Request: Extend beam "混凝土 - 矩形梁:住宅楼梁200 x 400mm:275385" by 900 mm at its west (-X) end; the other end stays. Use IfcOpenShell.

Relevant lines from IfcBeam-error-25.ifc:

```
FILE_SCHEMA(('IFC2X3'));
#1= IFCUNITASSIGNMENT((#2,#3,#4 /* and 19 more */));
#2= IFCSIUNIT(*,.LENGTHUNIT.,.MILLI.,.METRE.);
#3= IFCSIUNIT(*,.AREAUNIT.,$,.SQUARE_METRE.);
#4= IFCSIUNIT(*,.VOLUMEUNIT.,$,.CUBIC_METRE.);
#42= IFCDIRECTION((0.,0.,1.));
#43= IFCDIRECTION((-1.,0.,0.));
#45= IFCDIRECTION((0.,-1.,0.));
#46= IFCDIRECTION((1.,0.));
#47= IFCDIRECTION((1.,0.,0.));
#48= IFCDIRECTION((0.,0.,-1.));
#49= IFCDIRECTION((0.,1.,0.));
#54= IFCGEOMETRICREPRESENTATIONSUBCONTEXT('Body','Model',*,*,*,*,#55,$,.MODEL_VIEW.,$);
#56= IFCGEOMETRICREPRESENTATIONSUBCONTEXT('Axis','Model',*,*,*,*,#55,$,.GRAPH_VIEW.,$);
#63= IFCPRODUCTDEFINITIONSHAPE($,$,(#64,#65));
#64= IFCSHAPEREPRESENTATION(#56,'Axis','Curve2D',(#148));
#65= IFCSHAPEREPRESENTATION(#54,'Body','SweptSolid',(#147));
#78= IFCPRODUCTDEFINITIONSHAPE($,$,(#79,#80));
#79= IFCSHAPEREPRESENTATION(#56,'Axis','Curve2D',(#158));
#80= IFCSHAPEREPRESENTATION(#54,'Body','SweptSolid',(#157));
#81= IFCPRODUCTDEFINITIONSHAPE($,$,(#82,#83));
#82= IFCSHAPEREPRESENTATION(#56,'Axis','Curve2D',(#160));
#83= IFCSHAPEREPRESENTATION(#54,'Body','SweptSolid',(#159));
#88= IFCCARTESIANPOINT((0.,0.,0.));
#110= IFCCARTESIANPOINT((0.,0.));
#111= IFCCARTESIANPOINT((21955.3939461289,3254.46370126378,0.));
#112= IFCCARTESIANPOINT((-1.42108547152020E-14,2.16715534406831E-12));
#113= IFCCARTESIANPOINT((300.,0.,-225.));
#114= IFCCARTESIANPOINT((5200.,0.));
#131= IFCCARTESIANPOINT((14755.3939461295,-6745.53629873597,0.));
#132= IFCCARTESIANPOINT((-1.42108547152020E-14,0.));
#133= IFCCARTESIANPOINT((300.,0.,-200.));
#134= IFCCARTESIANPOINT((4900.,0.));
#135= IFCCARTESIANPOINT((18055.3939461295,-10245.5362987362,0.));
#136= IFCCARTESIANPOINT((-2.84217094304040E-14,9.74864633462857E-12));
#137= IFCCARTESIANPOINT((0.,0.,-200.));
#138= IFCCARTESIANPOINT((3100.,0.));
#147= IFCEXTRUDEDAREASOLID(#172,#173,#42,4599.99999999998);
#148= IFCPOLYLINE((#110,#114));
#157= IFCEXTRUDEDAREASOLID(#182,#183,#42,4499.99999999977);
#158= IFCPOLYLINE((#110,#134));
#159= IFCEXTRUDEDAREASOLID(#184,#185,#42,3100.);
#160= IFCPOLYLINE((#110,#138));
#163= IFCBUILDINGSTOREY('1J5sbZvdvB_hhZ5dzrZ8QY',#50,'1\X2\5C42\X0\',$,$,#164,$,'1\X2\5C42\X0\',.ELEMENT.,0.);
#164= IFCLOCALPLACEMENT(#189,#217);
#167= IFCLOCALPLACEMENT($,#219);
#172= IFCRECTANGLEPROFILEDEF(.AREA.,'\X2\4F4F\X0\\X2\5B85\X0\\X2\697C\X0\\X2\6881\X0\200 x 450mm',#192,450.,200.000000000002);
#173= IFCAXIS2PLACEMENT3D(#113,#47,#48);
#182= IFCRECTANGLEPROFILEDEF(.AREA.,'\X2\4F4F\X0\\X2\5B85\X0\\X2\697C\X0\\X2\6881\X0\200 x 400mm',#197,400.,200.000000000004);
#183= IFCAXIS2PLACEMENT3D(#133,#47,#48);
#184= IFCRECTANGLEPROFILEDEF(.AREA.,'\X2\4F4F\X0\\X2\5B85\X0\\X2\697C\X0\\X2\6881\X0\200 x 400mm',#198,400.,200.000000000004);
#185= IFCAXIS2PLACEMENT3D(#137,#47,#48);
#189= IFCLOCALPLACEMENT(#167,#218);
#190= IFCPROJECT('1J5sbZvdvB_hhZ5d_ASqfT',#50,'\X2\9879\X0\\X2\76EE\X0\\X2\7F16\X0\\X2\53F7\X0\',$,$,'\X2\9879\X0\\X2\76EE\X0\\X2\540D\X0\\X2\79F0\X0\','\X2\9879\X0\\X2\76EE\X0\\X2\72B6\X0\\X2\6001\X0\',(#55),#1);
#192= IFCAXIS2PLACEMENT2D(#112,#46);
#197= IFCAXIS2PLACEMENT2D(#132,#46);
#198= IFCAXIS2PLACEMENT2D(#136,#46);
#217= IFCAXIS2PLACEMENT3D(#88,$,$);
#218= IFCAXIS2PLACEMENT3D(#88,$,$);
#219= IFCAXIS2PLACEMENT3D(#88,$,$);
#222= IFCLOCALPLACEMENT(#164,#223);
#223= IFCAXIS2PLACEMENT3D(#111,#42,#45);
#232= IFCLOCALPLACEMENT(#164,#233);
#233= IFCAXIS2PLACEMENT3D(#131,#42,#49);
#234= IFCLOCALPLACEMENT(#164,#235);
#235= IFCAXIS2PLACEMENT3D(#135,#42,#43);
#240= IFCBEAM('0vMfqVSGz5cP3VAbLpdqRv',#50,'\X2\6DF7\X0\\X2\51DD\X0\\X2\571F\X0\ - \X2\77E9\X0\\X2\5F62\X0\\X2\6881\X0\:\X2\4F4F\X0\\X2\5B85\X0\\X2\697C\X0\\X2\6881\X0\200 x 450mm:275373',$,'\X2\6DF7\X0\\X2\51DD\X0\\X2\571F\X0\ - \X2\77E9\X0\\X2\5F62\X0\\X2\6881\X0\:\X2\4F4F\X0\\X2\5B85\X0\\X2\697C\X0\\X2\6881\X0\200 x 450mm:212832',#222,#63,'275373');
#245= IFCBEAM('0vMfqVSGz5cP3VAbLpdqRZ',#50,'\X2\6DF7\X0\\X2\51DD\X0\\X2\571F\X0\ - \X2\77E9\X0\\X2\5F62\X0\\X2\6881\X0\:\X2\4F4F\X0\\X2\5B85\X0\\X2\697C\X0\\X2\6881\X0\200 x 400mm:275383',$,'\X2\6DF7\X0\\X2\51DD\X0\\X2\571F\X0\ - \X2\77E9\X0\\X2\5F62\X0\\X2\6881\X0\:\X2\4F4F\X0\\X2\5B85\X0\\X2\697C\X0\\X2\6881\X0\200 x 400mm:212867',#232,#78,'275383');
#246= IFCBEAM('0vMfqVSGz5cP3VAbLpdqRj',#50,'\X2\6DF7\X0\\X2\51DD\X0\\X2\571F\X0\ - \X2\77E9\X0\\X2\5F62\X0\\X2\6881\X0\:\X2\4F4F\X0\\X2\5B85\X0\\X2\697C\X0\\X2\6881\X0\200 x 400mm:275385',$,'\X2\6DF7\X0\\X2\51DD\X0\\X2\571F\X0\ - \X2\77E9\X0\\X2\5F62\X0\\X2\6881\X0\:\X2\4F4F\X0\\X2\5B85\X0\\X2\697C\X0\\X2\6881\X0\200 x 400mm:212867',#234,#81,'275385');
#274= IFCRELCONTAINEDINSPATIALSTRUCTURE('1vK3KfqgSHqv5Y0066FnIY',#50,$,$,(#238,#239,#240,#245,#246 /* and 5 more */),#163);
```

```python
import numpy as np
import ifcopenshell
import ifcopenshell.util.representation

model = ifcopenshell.open("IfcBeam-error-25.ifc")

member = model.by_id(246)
change = 900.0

# The extrusion runs towards the end named, so only its depth changes.
body = ifcopenshell.util.representation.get_representation(member, "Model", "Body")
solid = body.Items[0]
old_length = solid.Depth
solid.Depth += change

# Move the axis end point with it.
axis = next(r for r in member.Representation.Representations if r.RepresentationIdentifier == "Axis").Items[0]
start, end = (np.array(p.Coordinates) for p in axis.Points)
end = end + (end - start) / np.linalg.norm(end - start) * change
point = model.createIfcCartesianPoint(end.tolist())
axis.Points = [axis.Points[0], point]

print(f"length {old_length:g} -> {solid.Depth:g}")

model.write("IfcBeam-error-25_rev.ifc")
```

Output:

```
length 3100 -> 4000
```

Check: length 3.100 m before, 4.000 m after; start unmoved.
